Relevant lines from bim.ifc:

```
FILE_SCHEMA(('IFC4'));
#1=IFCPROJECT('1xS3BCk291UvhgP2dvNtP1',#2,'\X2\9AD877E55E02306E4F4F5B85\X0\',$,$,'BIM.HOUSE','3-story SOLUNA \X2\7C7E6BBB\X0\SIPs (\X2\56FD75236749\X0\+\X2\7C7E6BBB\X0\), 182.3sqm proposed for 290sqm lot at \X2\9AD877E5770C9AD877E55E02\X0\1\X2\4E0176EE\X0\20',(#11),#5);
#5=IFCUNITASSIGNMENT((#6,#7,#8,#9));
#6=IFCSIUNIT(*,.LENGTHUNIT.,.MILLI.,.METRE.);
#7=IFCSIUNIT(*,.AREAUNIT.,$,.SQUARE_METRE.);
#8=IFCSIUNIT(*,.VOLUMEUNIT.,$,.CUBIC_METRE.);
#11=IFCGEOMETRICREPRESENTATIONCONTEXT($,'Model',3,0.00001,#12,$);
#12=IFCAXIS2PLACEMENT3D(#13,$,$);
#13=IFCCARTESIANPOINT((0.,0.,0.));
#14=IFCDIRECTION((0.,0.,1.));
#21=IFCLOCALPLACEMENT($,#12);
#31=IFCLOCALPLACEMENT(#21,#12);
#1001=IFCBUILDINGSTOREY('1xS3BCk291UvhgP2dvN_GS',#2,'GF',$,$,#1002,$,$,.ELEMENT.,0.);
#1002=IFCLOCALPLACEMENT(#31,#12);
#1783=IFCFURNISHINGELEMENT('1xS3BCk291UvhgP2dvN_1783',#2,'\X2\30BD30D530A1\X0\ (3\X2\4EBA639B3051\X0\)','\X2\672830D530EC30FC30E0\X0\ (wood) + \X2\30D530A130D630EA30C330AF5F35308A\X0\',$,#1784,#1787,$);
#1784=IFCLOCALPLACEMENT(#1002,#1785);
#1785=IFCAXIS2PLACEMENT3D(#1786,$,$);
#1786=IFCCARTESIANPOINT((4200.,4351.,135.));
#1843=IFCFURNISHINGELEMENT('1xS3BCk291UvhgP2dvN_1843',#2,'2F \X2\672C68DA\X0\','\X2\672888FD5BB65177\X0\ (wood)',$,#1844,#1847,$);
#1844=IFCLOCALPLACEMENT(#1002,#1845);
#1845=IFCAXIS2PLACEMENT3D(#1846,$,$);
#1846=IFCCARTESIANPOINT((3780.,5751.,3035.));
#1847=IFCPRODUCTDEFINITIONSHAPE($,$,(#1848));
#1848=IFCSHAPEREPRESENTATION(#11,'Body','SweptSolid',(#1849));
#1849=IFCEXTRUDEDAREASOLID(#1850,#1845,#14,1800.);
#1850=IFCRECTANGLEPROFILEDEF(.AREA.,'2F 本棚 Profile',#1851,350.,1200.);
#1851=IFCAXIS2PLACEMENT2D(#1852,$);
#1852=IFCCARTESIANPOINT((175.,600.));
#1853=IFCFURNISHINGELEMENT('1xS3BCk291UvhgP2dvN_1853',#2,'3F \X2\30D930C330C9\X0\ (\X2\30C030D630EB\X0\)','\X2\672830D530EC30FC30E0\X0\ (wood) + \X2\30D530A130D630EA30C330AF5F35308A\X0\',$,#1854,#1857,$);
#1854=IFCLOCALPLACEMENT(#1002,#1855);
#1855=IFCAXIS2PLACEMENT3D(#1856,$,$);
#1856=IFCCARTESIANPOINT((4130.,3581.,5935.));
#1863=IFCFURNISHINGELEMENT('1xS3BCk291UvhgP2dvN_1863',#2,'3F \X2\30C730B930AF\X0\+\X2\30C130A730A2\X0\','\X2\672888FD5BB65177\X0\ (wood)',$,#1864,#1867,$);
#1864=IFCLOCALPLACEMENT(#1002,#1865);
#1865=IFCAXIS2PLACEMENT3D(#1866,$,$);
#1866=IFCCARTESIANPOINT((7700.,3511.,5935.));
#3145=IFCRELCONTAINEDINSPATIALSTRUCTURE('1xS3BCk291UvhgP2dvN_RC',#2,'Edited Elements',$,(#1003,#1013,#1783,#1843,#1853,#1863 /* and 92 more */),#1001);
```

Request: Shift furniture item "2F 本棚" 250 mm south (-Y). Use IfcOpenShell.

```python
import ifcopenshell
import ifcopenshell.api.geometry
import ifcopenshell.util.placement

model = ifcopenshell.open("bim.ifc")

item = model.by_guid("1xS3BCk291UvhgP2dvN_1843")
matrix = ifcopenshell.util.placement.get_local_placement(item.ObjectPlacement)
matrix[1, 3] -= 250.0
ifcopenshell.api.geometry.edit_object_placement(model, product=item, matrix=matrix, is_si=False)

print(ifcopenshell.util.placement.get_local_placement(item.ObjectPlacement).round(3) + 0.0)

model.write("bim_v2.ifc")
```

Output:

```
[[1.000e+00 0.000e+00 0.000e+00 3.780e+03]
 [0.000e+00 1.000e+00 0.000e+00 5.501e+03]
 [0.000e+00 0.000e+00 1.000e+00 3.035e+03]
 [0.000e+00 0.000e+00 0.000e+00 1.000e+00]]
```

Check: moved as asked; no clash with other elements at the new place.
